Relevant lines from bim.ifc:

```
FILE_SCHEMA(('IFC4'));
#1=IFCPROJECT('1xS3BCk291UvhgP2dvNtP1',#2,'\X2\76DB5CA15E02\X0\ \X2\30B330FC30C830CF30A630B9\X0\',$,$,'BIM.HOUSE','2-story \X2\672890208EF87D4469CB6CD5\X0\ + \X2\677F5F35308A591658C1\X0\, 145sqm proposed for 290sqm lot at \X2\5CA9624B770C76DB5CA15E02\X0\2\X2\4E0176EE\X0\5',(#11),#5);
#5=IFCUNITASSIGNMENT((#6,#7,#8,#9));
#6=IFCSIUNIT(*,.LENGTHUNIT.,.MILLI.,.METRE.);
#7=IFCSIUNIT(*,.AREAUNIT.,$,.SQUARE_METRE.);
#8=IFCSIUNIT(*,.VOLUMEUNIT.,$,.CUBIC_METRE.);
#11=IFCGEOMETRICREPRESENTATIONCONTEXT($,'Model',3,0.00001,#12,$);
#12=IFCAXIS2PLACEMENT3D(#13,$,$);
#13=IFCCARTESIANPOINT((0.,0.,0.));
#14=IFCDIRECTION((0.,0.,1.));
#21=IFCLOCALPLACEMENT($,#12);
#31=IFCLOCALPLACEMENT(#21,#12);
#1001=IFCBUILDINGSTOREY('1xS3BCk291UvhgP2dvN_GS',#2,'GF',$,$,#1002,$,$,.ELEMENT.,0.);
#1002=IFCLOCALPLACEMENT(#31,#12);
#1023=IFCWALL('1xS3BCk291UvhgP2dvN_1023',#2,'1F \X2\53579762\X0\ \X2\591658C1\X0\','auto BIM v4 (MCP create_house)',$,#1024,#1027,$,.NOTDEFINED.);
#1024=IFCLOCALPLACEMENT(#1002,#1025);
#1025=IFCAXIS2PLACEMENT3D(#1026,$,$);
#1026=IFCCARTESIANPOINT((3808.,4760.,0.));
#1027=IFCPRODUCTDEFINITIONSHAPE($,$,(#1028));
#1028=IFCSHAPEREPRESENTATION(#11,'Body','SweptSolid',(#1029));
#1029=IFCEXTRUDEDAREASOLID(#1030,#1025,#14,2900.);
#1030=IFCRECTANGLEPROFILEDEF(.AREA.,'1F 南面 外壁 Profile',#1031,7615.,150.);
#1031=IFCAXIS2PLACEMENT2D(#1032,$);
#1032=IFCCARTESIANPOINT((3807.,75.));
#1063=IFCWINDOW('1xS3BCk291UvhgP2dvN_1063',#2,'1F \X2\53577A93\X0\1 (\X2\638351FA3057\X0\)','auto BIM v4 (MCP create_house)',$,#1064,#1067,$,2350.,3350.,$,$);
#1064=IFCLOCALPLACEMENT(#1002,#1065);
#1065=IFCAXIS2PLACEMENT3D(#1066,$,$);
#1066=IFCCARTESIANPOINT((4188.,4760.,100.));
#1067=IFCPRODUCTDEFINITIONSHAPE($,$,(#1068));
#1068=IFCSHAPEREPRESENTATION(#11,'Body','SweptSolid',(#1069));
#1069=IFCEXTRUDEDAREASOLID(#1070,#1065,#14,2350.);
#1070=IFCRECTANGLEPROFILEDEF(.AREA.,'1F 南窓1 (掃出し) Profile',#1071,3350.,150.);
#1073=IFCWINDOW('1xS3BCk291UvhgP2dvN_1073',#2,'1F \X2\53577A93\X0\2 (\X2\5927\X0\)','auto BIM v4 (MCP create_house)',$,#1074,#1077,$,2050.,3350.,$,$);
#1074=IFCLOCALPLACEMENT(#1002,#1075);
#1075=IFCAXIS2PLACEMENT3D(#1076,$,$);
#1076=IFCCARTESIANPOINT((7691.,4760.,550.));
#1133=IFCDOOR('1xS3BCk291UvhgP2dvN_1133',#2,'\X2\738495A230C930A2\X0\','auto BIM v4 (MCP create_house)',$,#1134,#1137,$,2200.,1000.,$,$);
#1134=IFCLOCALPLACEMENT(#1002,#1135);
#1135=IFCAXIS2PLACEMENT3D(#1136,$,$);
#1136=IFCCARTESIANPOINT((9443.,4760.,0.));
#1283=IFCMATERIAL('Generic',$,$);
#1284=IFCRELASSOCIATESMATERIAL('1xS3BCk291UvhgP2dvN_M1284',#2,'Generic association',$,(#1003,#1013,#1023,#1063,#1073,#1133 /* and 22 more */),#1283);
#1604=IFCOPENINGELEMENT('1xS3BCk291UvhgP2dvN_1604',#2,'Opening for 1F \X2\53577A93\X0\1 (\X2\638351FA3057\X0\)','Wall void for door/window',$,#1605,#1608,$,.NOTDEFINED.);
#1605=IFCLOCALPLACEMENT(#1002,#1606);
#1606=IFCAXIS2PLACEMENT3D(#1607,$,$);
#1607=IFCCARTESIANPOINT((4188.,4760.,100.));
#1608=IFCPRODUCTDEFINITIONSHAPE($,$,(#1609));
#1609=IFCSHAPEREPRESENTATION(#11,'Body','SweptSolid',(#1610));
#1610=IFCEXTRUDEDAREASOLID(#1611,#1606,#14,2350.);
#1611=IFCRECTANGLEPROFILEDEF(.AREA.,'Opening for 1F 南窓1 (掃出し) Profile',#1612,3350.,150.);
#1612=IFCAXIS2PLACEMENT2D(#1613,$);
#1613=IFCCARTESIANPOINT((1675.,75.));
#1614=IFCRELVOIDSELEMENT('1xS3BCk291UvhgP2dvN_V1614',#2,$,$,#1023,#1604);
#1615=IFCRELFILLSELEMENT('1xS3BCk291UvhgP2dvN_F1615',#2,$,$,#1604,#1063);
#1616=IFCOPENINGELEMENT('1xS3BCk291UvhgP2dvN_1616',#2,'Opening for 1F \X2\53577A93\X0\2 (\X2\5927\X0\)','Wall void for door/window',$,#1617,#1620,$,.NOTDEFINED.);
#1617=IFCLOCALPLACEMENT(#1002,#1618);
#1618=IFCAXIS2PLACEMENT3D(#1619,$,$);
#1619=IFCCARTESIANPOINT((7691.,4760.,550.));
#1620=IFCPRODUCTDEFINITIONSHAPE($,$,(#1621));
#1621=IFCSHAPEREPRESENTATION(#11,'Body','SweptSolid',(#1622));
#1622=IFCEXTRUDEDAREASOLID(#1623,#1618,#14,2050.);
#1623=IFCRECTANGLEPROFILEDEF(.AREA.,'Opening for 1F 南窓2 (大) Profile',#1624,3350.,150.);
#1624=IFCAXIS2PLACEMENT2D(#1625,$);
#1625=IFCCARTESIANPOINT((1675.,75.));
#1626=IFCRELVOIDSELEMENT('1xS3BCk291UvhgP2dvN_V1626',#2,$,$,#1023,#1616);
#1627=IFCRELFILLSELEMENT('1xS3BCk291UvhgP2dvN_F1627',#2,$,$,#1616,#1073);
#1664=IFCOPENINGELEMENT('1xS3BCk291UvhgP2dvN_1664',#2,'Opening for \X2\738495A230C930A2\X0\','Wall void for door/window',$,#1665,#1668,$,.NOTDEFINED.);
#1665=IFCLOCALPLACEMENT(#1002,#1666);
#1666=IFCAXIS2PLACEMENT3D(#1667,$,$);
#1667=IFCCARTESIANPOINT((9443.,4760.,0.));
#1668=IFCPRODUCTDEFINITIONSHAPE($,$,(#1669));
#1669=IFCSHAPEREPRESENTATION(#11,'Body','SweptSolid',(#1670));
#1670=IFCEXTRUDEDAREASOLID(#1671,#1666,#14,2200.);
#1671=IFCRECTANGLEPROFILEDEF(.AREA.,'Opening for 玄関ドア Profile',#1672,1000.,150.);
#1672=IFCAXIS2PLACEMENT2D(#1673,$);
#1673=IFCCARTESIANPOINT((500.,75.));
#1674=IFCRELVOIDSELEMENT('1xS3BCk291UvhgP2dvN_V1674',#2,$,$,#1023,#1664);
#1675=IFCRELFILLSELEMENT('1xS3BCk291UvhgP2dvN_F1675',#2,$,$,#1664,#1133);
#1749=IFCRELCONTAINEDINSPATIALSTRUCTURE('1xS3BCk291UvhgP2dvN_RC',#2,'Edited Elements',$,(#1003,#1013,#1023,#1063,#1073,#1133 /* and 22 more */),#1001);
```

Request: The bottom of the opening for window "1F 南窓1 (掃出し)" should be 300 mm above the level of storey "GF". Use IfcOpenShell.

```python
import numpy as np
import ifcopenshell
import ifcopenshell.api.geometry
import ifcopenshell.geom
import ifcopenshell.util.element
import ifcopenshell.util.placement
import ifcopenshell.util.shape
import ifcopenshell.util.unit

model = ifcopenshell.open("bim.ifc")
unit_scale = ifcopenshell.util.unit.calculate_unit_scale(model)

window = model.by_id(1063)
opening = window.FillsVoids[0].RelatingOpeningElement
storey = ifcopenshell.util.element.get_container(window, ifc_class="IfcBuildingStorey")
level = ifcopenshell.util.placement.get_local_placement(storey.ObjectPlacement)[2, 3]

# The opening's origin need not be at the sill, so measure its lowest point.
shape = ifcopenshell.geom.create_shape(ifcopenshell.geom.settings(), opening)
bottom = ifcopenshell.util.shape.get_shape_bottom_elevation(shape, shape.geometry) / unit_scale
dz = level + 300.0 - bottom

shift = np.array([0.0, 0.0, dz])
# The window is not placed relative to its opening, so move both.
for product in (opening, window):
    matrix = ifcopenshell.util.placement.get_local_placement(product.ObjectPlacement)
    matrix[:3, 3] += shift
    ifcopenshell.api.geometry.edit_object_placement(model, product=product, matrix=matrix, is_si=False)

print(f"moved by {dz * unit_scale:+.3f} m")

model.write("bim-out.ifc")
```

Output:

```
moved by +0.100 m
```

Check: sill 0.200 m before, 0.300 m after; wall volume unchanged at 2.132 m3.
